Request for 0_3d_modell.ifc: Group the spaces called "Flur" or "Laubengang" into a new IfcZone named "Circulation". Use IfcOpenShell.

First a look at what the model holds.

```python
import ifcopenshell

model = ifcopenshell.open("0_3d_modell.ifc")
print(model.schema)
seen = {}
for space in model.by_type("IfcSpace"):
    seen[space.LongName] = seen.get(space.LongName, 0) + 1
for name, count in sorted(seen.items(), key=str):
    print(count, "x", name)
print("zones:", [z.Name for z in model.by_type("IfcZone")][:20])
```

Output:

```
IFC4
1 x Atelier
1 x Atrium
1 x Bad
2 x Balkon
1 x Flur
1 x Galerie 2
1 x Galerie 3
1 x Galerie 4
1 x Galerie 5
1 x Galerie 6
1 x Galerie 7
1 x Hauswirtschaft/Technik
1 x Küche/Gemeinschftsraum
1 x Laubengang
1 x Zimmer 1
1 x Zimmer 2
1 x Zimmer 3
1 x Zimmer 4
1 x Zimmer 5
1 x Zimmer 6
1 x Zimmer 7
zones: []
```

```python
import ifcopenshell
import ifcopenshell.api.group
import ifcopenshell.api.root

model = ifcopenshell.open("0_3d_modell.ifc")

names = {"Flur", "Laubengang"}
spaces = [s for s in model.by_type("IfcSpace") if s.LongName in names]

zone = ifcopenshell.api.root.create_entity(model, ifc_class="IfcZone", name="Circulation")
ifcopenshell.api.group.assign_group(model, products=spaces, group=zone)
print(len(spaces), "spaces in", zone.Name)

model.write("0_3d_modell_rev.ifc")
```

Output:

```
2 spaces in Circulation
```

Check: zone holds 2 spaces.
